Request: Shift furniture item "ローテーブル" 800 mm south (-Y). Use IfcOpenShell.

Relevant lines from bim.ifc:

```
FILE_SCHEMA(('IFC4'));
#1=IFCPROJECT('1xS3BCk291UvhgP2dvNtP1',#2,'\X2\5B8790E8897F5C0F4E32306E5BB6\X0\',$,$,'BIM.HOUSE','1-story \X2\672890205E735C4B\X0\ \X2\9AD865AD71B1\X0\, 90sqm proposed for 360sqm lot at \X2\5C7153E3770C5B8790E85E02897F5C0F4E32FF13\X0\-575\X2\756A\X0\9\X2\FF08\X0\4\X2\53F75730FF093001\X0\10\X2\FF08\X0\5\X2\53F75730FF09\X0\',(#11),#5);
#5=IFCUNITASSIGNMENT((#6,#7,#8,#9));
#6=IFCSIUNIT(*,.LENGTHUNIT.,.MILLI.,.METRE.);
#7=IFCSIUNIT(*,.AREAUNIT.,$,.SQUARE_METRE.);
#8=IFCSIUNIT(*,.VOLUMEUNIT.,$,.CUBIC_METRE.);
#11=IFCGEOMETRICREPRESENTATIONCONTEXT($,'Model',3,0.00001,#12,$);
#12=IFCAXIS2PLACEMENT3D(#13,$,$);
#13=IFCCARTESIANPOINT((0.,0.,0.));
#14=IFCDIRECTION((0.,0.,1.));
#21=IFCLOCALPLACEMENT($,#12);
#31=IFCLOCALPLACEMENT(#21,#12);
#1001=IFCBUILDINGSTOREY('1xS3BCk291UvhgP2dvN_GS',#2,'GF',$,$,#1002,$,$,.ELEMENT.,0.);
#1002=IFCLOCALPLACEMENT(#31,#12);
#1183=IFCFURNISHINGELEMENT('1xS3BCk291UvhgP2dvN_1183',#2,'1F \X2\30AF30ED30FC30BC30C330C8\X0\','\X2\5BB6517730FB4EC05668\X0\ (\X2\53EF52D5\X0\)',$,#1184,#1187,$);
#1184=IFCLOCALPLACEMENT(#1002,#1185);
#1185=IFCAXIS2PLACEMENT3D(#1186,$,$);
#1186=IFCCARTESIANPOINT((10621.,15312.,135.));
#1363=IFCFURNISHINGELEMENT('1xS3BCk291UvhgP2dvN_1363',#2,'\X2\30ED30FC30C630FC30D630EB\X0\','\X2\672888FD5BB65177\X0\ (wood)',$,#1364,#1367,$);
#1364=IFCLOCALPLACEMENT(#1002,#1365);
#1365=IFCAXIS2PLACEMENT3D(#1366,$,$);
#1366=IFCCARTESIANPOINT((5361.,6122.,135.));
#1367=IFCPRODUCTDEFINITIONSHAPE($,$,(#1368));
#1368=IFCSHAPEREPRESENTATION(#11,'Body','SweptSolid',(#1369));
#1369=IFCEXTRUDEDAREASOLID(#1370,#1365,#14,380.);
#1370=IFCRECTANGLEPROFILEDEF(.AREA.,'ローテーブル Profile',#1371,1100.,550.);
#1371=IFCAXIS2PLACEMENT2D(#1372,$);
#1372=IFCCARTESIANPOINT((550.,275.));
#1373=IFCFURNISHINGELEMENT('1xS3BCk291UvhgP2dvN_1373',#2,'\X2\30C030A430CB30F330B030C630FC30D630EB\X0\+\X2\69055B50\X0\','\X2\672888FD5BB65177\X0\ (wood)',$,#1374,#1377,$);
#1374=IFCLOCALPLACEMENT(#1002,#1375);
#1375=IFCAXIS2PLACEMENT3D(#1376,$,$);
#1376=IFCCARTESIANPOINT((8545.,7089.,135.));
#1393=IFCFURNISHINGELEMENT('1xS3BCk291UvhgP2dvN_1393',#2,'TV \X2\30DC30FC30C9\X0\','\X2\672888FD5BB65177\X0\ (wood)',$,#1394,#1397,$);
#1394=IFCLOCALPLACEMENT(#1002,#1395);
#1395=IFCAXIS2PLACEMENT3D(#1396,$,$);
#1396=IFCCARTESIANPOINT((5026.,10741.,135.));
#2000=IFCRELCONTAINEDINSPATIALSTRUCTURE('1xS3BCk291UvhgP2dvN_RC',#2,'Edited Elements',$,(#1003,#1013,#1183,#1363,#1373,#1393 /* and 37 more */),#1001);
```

```python
import ifcopenshell
import ifcopenshell.api.geometry
import ifcopenshell.util.placement
import ifcopenshell.util.unit

model = ifcopenshell.open("bim.ifc")
unit_scale = ifcopenshell.util.unit.calculate_unit_scale(model)

item = model.by_guid("1xS3BCk291UvhgP2dvN_1363")
matrix = ifcopenshell.util.placement.get_local_placement(item.ObjectPlacement)
matrix[1, 3] -= 0.8 / unit_scale
ifcopenshell.api.geometry.edit_object_placement(model, product=item, matrix=matrix, is_si=False)

print(ifcopenshell.util.placement.get_local_placement(item.ObjectPlacement).round(3) + 0.0)

model.write("bim_v2.ifc")
```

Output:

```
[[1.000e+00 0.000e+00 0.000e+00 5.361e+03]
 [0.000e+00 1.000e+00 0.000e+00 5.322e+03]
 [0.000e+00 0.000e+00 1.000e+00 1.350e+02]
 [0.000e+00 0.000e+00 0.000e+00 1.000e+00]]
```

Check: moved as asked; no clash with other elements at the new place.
